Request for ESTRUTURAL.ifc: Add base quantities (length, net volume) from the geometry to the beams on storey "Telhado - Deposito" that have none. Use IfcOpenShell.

First a look at what the model holds.

```python
import ifcopenshell
import ifcopenshell.util.element
import ifcopenshell.util.unit

model = ifcopenshell.open("ESTRUTURAL.ifc")
print(model.schema)
for unit_type in ("LENGTHUNIT", "AREAUNIT", "VOLUMEUNIT"):
    print(unit_type, ifcopenshell.util.unit.calculate_unit_scale(model, unit_type))
storey = next(s for s in model.by_type("IfcBuildingStorey") if s.Name == "Telhado - Deposito")
beams = [e for e in ifcopenshell.util.element.get_decomposition(storey) if e.is_a("IfcBeam")]
for e in sorted(beams, key=lambda e: e.id()):
    print(e.id(), e.is_a(), e.Name, list(ifcopenshell.util.element.get_psets(e, qtos_only=True)), sep=" | ")
```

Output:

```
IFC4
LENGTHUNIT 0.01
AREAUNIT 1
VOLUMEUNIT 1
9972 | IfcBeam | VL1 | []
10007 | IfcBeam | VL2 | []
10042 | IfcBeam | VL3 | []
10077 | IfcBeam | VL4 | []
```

```python
import ifcopenshell
import ifcopenshell.api.pset
import ifcopenshell.geom
import ifcopenshell.util.element
import ifcopenshell.util.shape
import ifcopenshell.util.unit

model = ifcopenshell.open("ESTRUTURAL.ifc")
unit_scale = ifcopenshell.util.unit.calculate_unit_scale(model)
volume_scale = ifcopenshell.util.unit.calculate_unit_scale(model, "VOLUMEUNIT")
settings = ifcopenshell.geom.settings()

storey = next(s for s in model.by_type("IfcBuildingStorey") if s.Name == "Telhado - Deposito")
beams = [e for e in ifcopenshell.util.element.get_decomposition(storey) if e.is_a("IfcBeam")]

for e in sorted(beams, key=lambda e: e.id()):
    if ifcopenshell.util.element.get_psets(e, qtos_only=True, should_inherit=False):
        continue
    # Geometry comes back in metres, in the element's own axes.
    shape = ifcopenshell.geom.create_shape(settings, e)
    values = {
        "Length": ifcopenshell.util.shape.get_max_xyz(shape.geometry) / unit_scale,
        "NetVolume": ifcopenshell.util.shape.get_volume(shape.geometry) / volume_scale,
    }
    qto = ifcopenshell.api.pset.add_qto(model, product=e, name="Qto_BeamBaseQuantities")
    ifcopenshell.api.pset.edit_qto(model, qto=qto, properties=values)
    print(e.id(), {k: round(v, 3) for k, v in values.items()})

model.write("ESTRUTURAL-out.ifc")
```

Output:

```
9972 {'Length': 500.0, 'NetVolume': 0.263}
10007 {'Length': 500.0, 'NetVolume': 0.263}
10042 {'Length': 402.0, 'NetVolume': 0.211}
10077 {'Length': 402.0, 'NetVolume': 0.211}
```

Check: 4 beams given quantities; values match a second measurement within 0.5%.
